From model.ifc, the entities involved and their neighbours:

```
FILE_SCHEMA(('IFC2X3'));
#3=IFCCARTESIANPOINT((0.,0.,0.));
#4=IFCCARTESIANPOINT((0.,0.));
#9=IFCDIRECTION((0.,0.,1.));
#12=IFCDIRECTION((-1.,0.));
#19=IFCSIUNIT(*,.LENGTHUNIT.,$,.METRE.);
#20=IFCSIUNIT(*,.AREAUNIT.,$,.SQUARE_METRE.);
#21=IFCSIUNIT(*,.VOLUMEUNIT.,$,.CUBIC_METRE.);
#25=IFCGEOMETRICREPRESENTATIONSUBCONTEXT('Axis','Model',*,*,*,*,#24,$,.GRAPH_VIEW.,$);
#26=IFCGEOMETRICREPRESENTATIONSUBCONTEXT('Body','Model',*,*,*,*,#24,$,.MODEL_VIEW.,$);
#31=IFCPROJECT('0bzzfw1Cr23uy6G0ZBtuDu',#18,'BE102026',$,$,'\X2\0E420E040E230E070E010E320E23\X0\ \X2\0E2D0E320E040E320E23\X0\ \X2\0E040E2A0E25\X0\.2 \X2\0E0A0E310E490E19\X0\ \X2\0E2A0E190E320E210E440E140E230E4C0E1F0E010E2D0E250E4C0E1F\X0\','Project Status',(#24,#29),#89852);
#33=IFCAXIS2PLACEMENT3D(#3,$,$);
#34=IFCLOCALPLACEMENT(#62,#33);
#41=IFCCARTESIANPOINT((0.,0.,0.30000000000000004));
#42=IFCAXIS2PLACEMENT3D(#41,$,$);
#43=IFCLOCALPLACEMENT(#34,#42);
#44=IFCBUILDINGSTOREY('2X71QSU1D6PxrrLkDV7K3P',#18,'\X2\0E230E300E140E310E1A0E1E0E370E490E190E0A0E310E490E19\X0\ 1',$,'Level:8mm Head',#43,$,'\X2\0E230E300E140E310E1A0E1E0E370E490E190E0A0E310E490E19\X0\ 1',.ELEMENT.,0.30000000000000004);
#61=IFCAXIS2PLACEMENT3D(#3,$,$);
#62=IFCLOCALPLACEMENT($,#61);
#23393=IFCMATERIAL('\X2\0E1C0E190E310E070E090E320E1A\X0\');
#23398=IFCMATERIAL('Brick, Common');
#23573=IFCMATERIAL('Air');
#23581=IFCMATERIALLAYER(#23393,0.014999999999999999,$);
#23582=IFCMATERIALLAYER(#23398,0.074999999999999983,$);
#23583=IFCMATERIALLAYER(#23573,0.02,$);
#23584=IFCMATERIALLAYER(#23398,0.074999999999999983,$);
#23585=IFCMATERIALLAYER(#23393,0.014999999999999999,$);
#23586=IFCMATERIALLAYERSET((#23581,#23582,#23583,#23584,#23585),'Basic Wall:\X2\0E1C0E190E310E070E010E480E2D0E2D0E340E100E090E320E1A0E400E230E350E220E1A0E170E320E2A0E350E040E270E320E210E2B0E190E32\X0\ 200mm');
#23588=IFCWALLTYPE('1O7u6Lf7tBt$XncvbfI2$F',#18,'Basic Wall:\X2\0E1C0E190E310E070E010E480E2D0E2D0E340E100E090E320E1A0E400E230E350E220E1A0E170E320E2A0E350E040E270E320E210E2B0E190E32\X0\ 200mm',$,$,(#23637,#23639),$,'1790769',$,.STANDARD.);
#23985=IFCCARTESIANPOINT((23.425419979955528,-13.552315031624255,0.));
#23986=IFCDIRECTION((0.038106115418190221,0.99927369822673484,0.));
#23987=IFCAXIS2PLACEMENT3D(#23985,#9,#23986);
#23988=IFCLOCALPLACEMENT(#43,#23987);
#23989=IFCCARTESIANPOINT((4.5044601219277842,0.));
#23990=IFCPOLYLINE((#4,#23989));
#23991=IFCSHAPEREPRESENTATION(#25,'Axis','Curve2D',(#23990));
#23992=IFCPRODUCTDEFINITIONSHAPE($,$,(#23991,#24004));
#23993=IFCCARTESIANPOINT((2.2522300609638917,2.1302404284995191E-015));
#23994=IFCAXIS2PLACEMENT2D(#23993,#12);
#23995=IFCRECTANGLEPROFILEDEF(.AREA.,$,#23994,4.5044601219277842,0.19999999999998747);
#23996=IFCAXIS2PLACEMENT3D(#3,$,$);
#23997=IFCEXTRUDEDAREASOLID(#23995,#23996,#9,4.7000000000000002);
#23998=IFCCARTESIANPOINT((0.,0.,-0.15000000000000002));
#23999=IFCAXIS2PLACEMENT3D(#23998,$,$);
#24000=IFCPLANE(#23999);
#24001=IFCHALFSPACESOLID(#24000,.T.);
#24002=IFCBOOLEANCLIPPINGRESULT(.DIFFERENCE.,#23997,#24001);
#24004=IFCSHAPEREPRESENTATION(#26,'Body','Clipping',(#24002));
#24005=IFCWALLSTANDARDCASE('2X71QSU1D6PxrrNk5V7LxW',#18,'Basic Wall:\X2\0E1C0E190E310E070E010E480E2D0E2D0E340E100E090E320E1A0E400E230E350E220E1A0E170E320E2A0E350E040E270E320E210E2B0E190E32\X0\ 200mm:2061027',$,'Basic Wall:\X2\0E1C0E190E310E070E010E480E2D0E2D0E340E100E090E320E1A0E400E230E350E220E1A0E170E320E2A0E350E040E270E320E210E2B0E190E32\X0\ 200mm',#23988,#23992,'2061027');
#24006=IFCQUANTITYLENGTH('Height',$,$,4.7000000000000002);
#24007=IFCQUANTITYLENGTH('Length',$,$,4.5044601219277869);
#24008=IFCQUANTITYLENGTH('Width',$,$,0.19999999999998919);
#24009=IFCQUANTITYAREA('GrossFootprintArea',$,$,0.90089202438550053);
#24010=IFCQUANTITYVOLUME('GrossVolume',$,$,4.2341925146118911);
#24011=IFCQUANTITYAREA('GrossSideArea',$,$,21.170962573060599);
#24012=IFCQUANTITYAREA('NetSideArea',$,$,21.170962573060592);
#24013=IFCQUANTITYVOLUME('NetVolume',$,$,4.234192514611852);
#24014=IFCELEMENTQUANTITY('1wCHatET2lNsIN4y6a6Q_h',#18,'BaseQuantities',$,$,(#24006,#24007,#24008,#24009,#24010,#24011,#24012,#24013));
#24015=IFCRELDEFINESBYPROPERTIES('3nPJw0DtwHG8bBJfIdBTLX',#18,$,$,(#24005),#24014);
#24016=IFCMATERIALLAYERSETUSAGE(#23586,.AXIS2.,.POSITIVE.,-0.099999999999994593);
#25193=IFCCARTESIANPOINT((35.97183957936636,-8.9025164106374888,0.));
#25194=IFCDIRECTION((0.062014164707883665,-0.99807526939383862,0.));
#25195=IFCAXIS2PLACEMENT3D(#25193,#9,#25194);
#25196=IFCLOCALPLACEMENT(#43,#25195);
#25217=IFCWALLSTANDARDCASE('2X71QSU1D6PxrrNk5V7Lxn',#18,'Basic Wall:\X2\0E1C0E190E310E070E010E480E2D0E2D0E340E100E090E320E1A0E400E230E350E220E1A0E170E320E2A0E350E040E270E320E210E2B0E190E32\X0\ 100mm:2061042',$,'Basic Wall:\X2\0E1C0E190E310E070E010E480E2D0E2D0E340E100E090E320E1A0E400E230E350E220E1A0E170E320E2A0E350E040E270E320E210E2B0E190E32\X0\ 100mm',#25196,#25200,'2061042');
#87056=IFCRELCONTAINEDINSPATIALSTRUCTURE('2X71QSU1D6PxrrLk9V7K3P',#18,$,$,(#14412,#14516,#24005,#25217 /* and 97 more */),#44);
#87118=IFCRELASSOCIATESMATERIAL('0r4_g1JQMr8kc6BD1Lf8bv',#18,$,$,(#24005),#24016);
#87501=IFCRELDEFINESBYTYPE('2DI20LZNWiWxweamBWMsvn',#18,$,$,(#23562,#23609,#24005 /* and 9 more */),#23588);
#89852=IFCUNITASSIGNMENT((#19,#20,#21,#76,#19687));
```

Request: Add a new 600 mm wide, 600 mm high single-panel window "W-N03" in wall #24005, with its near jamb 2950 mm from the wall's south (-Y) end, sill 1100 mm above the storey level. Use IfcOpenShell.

```python
import numpy as np
import ifcopenshell
import ifcopenshell.api.feature
import ifcopenshell.api.geometry
import ifcopenshell.api.pset
import ifcopenshell.api.root
import ifcopenshell.api.spatial
import ifcopenshell.api.type
import ifcopenshell.geom
import ifcopenshell.util.element
import ifcopenshell.util.placement
import ifcopenshell.util.representation
import ifcopenshell.util.shape
import ifcopenshell.util.unit

model = ifcopenshell.open("model.ifc")
unit_scale = ifcopenshell.util.unit.calculate_unit_scale(model)
area_scale = ifcopenshell.util.unit.calculate_unit_scale(model, "AREAUNIT")
volume_scale = ifcopenshell.util.unit.calculate_unit_scale(model, "VOLUMEUNIT")
settings = ifcopenshell.geom.settings()


def volume(element):
    """Net volume in cubic metres, openings subtracted."""
    shape = ifcopenshell.geom.create_shape(settings, element)
    return ifcopenshell.util.shape.get_volume(shape.geometry)


wall = model.by_guid("2X71QSU1D6PxrrNk5V7LxW")
storey = ifcopenshell.util.element.get_container(wall, ifc_class="IfcBuildingStorey")
context = ifcopenshell.util.representation.get_context(model, "Model", "Body", "MODEL_VIEW")
before = volume(wall)

width, height, from_end, sill = 0.6, 0.6, 2.95, 1.1  # metres

# The wall runs along its own X axis, and the end named is its -X end.
wall_shape = ifcopenshell.geom.create_shape(settings, wall)
x, y, z = ifcopenshell.util.shape.get_vertices(wall_shape.geometry).T
start = x.min() + from_end
face, thickness = float(y.min()), float(y.max() - y.min())
wall_matrix = ifcopenshell.util.placement.get_local_placement(wall.ObjectPlacement)
level = ifcopenshell.util.placement.get_local_placement(storey.ObjectPlacement)[2, 3]


def in_wall(x, y):
    """Placement at x, y metres in the wall's axes, at sill height."""
    matrix = wall_matrix.copy()
    matrix[:, 3] = wall_matrix @ np.array([x / unit_scale, y / unit_scale, 0.0, 1.0])
    matrix[2, 3] = level + sill / unit_scale
    return matrix


# Opening: a box that overshoots both wall faces by 50 mm.
opening = ifcopenshell.api.root.create_entity(model, ifc_class="IfcOpeningElement")
box = ifcopenshell.api.geometry.add_wall_representation(
    model, context=context, length=width, height=height, thickness=thickness + 0.1
)
ifcopenshell.api.geometry.assign_representation(model, product=opening, representation=box)
ifcopenshell.api.geometry.edit_object_placement(model, product=opening, matrix=in_wall(start, face - 0.05), is_si=False)
ifcopenshell.api.feature.add_feature(model, feature=opening, element=wall)

window = ifcopenshell.api.root.create_entity(model, ifc_class="IfcWindow", name="W-N03")
window.OverallWidth, window.OverallHeight = width / unit_scale, height / unit_scale
body = ifcopenshell.api.geometry.add_window_representation(
    model,
    context=context,
    overall_width=window.OverallWidth,
    overall_height=window.OverallHeight,
    partition_type="SINGLE_PANEL",
)
ifcopenshell.api.geometry.assign_representation(model, product=window, representation=body)
ifcopenshell.api.spatial.assign_container(model, products=[window], relating_structure=storey)
fills = ifcopenshell.api.feature.add_filling(model, opening=opening, element=window)
fills.OwnerHistory = window.OwnerHistory  # required in IFC2X3

# IFC2X3 keeps the operation on the window style.
style = ifcopenshell.api.root.create_entity(model, ifc_class="IfcWindowStyle", name="W-N03")
style.OperationType, style.ConstructionType = "SINGLE_PANEL", "NOTDEFINED"
style.ParameterTakesPrecedence = style.Sizeable = False
ifcopenshell.api.type.assign_type(model, related_objects=[window], relating_type=style)

# Centre the window in the wall's thickness.
ifcopenshell.api.geometry.edit_object_placement(model, product=window, matrix=in_wall(start, face), is_si=False)
window_shape = ifcopenshell.geom.create_shape(settings, window)
depth = ifcopenshell.util.shape.get_vertices(window_shape.geometry)[:, 1]
offset = face + thickness / 2 - (depth.min() + depth.max()) / 2
ifcopenshell.api.geometry.edit_object_placement(model, product=window, matrix=in_wall(start, offset), is_si=False)

after = volume(wall)

# Update the wall's stored quantities.
qto = model.by_id(ifcopenshell.util.element.get_pset(wall, "BaseQuantities", should_inherit=False)["id"])
ifcopenshell.api.pset.edit_qto(model, qto=qto, properties={
    "NetSideArea": after / thickness / area_scale,
    "NetVolume": after / volume_scale,
})

print(f"wall volume {before:.3f} -> {after:.3f} m3")

model.write("model-out.ifc")
```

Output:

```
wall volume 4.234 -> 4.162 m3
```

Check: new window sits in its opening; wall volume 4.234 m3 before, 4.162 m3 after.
